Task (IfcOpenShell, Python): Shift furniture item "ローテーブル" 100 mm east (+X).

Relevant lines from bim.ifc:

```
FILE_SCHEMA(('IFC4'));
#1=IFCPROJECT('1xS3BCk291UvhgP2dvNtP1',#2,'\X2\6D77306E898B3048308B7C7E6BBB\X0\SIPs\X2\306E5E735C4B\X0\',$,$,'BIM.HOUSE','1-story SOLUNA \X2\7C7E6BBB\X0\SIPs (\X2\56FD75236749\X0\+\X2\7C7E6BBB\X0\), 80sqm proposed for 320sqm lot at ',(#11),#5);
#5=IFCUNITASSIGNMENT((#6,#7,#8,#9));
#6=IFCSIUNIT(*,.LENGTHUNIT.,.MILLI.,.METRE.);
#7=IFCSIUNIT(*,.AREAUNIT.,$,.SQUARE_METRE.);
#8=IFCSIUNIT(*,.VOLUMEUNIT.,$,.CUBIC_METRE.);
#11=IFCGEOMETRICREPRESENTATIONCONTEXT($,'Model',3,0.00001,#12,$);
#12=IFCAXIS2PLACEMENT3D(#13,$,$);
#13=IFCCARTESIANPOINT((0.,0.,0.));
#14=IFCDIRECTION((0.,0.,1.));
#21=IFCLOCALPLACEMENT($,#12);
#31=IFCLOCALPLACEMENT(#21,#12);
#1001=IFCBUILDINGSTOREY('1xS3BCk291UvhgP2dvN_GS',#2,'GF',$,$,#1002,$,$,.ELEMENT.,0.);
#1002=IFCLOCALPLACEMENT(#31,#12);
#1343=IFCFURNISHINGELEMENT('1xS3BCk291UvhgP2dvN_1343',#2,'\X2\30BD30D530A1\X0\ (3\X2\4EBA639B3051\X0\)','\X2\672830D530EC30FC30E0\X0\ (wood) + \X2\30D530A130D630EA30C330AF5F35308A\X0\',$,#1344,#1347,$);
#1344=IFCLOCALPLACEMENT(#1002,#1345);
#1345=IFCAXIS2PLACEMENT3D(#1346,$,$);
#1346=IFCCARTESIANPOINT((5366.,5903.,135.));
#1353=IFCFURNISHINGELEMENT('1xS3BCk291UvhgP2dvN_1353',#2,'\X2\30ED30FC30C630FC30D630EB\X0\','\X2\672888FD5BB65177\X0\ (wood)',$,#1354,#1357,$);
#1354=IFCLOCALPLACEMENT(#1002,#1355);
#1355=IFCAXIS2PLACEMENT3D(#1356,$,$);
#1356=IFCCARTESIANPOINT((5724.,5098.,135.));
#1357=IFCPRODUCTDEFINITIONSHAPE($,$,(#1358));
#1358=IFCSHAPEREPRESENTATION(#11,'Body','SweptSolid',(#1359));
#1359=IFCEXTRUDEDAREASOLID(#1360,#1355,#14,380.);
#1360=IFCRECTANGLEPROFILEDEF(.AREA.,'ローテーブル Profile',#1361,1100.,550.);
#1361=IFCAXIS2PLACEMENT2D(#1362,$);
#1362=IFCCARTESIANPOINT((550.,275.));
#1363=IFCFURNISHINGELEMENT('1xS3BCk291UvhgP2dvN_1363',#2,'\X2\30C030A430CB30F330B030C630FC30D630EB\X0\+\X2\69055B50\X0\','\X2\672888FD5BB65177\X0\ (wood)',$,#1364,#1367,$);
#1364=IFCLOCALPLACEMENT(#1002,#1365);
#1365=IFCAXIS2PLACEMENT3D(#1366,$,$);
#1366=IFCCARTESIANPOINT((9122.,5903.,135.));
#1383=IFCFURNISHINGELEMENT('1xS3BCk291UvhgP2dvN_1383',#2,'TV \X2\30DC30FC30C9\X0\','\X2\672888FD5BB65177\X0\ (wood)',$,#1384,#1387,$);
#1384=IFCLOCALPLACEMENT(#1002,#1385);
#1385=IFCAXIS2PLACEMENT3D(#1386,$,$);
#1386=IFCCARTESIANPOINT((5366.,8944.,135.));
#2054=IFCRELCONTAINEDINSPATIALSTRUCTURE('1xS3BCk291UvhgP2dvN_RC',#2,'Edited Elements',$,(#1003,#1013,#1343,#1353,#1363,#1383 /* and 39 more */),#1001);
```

```python
import ifcopenshell
import ifcopenshell.api.geometry
import ifcopenshell.util.placement
import ifcopenshell.util.unit

model = ifcopenshell.open("bim.ifc")
unit_scale = ifcopenshell.util.unit.calculate_unit_scale(model)

item = model.by_guid("1xS3BCk291UvhgP2dvN_1353")
matrix = ifcopenshell.util.placement.get_local_placement(item.ObjectPlacement)
matrix[0, 3] += 0.1 / unit_scale
ifcopenshell.api.geometry.edit_object_placement(model, product=item, matrix=matrix, is_si=False)

print(ifcopenshell.util.placement.get_local_placement(item.ObjectPlacement).round(3) + 0.0)

model.write("bim_rev.ifc")
```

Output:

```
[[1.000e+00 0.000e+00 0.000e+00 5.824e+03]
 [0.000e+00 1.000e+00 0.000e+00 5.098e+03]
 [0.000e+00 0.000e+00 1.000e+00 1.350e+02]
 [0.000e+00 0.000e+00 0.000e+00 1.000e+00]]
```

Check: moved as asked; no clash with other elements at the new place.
